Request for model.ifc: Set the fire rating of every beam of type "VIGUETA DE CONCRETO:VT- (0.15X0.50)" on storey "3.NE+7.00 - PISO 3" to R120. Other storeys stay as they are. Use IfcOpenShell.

First a look at what the model holds.

```python
import ifcopenshell
import ifcopenshell.util.element

model = ifcopenshell.open("model.ifc")
print(model.schema)
storey = next(s for s in model.by_type("IfcBuildingStorey") if s.Name == "3.NE+7.00 - PISO 3")
beams = [e for e in ifcopenshell.util.element.get_decomposition(storey) if e.is_a("IfcBeam")]
seen = {}
for e in beams:
    element_type = ifcopenshell.util.element.get_type(e)
    key = (element_type.Name if element_type != e and element_type else None, ifcopenshell.util.element.get_pset(e, "Pset_BeamCommon", "FireRating"))
    seen[key] = seen.get(key, 0) + 1
for (name, value), count in sorted(seen.items(), key=str):
    print(count, "x", name, "|", value)
```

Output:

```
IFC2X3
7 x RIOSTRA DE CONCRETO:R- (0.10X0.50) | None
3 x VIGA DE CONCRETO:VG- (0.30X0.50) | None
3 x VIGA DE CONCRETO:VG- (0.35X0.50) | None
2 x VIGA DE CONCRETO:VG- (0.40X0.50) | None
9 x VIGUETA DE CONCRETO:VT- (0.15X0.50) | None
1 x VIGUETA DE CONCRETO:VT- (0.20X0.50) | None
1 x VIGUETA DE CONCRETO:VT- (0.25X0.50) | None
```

```python
import ifcopenshell
import ifcopenshell.api.pset
import ifcopenshell.util.element

model = ifcopenshell.open("model.ifc")

storey = next(s for s in model.by_type("IfcBuildingStorey") if s.Name == "3.NE+7.00 - PISO 3")
beams = [e for e in ifcopenshell.util.element.get_decomposition(storey) if e.is_a("IfcBeam")]

count = 0
for e in beams:
    element_type = ifcopenshell.util.element.get_type(e)
    if element_type in (None, e) or element_type.Name != "VIGUETA DE CONCRETO:VT- (0.15X0.50)":
        continue
    # add_pset returns the element's existing set when there is one.
    pset = ifcopenshell.api.pset.add_pset(model, product=e, name="Pset_BeamCommon")
    ifcopenshell.api.pset.edit_pset(model, pset=pset, properties={"FireRating": "R120"})
    count += 1

print(count, "beams updated")

model.write("model_updated.ifc")
```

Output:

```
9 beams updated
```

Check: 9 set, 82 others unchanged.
